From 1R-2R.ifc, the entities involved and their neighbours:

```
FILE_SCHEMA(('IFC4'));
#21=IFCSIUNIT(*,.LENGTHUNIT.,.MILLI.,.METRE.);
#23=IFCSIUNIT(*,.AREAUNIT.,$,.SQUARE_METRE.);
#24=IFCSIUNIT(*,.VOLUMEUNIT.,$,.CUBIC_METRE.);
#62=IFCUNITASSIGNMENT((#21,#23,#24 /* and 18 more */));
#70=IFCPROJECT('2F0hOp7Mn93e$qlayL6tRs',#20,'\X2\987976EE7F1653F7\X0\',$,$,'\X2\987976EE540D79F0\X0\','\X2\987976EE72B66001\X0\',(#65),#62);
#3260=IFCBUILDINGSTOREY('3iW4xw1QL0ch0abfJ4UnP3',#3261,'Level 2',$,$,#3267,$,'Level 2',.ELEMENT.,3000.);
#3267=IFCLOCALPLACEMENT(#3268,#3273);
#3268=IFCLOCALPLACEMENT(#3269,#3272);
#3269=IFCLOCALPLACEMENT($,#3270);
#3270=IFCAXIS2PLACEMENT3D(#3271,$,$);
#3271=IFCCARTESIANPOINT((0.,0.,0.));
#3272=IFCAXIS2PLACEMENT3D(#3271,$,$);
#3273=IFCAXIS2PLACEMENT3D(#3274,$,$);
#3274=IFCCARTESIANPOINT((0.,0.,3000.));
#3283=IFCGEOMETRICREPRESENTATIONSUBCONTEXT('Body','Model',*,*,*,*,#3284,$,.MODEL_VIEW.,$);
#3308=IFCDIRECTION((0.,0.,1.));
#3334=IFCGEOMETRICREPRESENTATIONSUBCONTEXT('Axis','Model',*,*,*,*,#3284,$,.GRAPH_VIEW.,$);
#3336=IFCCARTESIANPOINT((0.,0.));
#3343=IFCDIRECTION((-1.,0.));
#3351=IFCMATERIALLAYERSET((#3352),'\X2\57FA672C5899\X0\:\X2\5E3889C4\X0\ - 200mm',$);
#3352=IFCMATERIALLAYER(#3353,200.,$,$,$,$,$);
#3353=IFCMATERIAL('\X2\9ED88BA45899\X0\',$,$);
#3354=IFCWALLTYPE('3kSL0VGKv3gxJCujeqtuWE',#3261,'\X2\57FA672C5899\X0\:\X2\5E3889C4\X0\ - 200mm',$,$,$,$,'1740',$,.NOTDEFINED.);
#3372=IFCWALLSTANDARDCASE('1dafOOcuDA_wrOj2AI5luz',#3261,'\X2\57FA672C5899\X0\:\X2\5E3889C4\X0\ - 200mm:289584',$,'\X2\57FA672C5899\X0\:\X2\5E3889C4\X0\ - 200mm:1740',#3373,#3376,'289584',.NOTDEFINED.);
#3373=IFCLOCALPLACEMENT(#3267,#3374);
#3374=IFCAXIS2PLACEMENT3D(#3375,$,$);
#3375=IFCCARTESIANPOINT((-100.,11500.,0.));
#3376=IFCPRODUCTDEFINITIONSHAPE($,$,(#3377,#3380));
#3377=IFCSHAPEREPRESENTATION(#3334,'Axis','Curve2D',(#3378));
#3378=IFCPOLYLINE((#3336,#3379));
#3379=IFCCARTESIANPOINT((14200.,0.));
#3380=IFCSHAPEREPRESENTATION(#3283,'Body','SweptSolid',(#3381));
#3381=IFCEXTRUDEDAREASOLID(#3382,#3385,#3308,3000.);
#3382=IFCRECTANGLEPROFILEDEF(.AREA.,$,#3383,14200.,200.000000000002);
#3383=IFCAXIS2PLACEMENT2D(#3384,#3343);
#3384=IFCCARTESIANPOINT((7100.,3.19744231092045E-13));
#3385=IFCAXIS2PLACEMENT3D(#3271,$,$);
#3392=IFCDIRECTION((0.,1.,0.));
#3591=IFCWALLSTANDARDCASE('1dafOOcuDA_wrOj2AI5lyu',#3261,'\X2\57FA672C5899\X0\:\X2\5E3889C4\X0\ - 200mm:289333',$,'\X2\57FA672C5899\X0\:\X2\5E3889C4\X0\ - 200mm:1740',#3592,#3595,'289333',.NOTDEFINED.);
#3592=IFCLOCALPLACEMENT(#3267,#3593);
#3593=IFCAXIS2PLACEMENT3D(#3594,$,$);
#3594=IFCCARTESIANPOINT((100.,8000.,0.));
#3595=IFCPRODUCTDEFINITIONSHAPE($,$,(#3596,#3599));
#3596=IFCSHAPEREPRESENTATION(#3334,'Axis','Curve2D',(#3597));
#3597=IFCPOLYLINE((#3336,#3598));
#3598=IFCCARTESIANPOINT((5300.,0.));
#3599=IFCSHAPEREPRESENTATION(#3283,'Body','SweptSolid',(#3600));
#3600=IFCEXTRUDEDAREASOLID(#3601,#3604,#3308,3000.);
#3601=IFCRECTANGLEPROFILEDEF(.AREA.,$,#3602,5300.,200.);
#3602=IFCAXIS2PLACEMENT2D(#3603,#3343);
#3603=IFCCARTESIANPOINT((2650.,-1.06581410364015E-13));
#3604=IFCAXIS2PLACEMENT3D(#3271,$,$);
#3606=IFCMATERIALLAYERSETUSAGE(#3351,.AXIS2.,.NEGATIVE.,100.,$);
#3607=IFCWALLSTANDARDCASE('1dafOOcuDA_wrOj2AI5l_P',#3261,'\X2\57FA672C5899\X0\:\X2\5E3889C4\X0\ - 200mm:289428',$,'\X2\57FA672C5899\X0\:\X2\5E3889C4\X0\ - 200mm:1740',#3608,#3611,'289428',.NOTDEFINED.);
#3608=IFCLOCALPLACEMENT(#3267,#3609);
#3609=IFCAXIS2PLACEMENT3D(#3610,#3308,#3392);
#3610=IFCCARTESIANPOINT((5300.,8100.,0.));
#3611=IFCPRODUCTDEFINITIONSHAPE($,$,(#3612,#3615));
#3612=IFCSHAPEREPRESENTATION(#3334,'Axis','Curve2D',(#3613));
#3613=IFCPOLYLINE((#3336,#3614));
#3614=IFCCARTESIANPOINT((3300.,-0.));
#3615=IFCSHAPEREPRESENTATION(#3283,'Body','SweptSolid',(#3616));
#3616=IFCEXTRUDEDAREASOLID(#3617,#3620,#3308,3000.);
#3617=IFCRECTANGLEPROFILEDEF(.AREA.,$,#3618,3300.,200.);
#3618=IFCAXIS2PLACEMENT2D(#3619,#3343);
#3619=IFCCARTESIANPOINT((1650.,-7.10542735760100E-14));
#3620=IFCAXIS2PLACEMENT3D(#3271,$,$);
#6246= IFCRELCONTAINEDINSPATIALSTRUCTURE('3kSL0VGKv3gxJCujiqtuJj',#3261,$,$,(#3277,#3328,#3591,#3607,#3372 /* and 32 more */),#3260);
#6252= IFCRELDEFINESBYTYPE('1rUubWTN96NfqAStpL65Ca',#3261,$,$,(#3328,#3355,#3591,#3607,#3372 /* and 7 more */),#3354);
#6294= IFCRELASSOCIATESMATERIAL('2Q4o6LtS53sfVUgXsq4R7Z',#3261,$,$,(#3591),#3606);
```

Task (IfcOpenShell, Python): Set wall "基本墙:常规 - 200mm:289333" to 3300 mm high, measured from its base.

```python
import ifcopenshell
import ifcopenshell.geom
import ifcopenshell.util.representation
import ifcopenshell.util.shape
import ifcopenshell.util.unit

model = ifcopenshell.open("1R-2R.ifc")
unit_scale = ifcopenshell.util.unit.calculate_unit_scale(model)
settings = ifcopenshell.geom.settings()


def volume(element):
    """Net volume in cubic metres, openings subtracted."""
    shape = ifcopenshell.geom.create_shape(settings, element)
    return ifcopenshell.util.shape.get_volume(shape.geometry)


wall = model.by_guid("1dafOOcuDA_wrOj2AI5lyu")
before = volume(wall)

body = ifcopenshell.util.representation.get_representation(wall, "Model", "Body")
solid = body.Items[0]
old_height = solid.Depth
solid.Depth = 3.3 / unit_scale
after = volume(wall)

print(f"height {old_height:g} -> {solid.Depth:g}, volume {before:.3f} -> {after:.3f} m3")

model.write("1R-2R_rev.ifc")
```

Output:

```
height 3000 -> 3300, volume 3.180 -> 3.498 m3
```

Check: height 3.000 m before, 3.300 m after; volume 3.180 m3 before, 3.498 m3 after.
